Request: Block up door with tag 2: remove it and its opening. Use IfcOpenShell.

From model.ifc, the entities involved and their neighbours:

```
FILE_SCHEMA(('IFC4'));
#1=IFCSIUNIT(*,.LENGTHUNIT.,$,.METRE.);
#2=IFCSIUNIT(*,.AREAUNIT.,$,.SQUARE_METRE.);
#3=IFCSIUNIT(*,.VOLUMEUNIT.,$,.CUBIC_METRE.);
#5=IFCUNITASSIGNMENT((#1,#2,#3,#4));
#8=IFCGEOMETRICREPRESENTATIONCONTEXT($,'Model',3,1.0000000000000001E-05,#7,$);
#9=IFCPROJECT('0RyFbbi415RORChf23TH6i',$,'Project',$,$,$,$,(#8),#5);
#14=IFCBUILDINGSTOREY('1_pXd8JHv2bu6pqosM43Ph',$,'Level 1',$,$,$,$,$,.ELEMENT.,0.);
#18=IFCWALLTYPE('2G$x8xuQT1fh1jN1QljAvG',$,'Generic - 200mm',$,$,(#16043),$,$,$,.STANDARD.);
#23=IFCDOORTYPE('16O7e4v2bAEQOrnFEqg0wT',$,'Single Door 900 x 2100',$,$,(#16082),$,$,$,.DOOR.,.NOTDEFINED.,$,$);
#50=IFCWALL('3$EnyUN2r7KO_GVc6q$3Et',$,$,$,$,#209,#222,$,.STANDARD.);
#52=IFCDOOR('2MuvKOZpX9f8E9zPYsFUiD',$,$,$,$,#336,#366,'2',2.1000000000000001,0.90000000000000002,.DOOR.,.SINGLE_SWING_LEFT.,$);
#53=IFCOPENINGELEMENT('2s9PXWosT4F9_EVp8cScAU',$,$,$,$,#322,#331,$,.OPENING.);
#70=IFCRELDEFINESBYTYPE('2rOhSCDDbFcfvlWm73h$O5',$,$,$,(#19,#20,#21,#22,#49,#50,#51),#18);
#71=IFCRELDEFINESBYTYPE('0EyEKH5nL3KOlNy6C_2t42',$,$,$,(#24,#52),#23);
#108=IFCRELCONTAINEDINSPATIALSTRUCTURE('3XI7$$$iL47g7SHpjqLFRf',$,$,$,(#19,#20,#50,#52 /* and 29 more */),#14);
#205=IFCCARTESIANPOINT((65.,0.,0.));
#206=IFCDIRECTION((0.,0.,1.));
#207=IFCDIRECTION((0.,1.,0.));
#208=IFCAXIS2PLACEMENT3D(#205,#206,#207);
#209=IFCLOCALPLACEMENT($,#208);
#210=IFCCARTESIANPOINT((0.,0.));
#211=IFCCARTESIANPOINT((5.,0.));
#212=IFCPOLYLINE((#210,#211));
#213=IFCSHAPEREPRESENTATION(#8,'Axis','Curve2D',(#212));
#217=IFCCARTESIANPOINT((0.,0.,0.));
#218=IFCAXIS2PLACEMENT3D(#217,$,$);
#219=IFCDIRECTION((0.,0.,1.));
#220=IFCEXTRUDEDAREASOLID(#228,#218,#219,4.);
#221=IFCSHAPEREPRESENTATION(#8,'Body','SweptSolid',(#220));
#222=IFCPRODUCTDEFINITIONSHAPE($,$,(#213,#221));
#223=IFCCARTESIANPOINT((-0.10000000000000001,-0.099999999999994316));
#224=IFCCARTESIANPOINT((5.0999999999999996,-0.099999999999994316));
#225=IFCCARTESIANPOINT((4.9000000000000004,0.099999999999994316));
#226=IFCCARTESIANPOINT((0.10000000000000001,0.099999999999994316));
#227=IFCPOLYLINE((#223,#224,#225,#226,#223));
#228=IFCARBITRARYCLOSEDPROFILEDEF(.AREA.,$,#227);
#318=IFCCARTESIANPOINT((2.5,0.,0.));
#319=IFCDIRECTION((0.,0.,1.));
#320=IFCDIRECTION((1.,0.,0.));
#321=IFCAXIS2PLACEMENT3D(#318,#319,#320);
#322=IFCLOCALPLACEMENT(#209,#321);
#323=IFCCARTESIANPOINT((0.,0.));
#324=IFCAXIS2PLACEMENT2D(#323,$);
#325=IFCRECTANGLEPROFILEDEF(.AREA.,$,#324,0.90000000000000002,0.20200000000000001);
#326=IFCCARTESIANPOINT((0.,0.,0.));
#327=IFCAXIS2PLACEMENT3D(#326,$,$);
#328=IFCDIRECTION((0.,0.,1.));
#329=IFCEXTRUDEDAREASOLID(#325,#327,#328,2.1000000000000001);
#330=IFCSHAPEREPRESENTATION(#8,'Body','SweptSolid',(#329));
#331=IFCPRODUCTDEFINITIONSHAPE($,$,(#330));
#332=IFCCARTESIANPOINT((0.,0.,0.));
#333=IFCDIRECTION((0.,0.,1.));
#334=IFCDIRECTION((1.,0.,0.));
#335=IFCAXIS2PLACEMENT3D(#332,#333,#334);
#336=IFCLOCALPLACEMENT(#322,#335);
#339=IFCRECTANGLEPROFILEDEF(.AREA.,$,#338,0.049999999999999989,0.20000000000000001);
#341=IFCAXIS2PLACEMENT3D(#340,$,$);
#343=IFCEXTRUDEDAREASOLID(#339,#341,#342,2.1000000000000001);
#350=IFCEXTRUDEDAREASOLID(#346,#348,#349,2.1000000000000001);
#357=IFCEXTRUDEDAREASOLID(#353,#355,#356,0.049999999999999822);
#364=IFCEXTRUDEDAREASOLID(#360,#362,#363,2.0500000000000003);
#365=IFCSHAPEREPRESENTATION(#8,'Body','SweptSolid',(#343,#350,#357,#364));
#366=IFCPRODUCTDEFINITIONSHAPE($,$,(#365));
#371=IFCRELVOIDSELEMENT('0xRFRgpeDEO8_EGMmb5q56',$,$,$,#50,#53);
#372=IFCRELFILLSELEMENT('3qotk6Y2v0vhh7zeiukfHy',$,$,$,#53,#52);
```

```python
import ifcopenshell
import ifcopenshell.api.feature
import ifcopenshell.api.root
import ifcopenshell.geom
import ifcopenshell.util.shape

model = ifcopenshell.open("model.ifc")
settings = ifcopenshell.geom.settings()


def volume(element):
    """Net volume in cubic metres, openings subtracted."""
    shape = ifcopenshell.geom.create_shape(settings, element)
    return ifcopenshell.util.shape.get_volume(shape.geometry)


door = model.by_guid("2MuvKOZpX9f8E9zPYsFUiD")
opening = door.FillsVoids[0].RelatingOpeningElement
wall = opening.VoidsElements[0].RelatingBuildingElement
before = volume(wall)

ifcopenshell.api.root.remove_product(model, product=door)
ifcopenshell.api.feature.remove_feature(model, feature=opening)

after = volume(wall)

print(f"wall volume {before:.3f} -> {after:.3f} m3")

model.write("model_v2.ifc")
```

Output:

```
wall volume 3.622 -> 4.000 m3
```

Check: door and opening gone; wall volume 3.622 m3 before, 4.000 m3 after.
